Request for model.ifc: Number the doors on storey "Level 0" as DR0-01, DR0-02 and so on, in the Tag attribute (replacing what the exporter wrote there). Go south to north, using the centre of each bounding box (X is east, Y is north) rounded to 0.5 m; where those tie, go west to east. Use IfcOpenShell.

First a look at what the model holds.

```python
import ifcopenshell
import ifcopenshell.util.element
import ifcopenshell.util.placement

model = ifcopenshell.open("model.ifc")
print(model.schema)
storey = next(s for s in model.by_type("IfcBuildingStorey") if s.Name == "Level 0")
doors = [e for e in ifcopenshell.util.element.get_decomposition(storey) if e.is_a("IfcDoor")]
for e in sorted(doors, key=lambda e: e.id()):
    origin = ifcopenshell.util.placement.get_local_placement(e.ObjectPlacement)[:3, 3]
    print(e.id(), e.Tag, e.Name, origin.round(2) + 0.0, sep=" | ")
```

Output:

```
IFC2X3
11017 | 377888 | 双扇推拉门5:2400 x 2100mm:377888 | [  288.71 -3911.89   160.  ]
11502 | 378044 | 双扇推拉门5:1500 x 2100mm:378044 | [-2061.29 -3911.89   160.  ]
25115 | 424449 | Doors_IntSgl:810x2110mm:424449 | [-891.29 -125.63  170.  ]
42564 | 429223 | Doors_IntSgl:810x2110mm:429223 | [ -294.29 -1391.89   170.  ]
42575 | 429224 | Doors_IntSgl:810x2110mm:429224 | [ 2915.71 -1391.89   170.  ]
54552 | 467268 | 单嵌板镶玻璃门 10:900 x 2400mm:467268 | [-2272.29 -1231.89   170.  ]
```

```python
import ifcopenshell
import ifcopenshell.geom
import ifcopenshell.util.element
import ifcopenshell.util.shape

model = ifcopenshell.open("model.ifc")
settings = ifcopenshell.geom.settings()
settings.set("use-world-coords", True)


def centre(element):
    shape = ifcopenshell.geom.create_shape(settings, element)
    return ifcopenshell.util.shape.get_bbox_centroid(shape.geometry)


storey = next(s for s in model.by_type("IfcBuildingStorey") if s.Name == "Level 0")
doors = [e for e in ifcopenshell.util.element.get_decomposition(storey) if e.is_a("IfcDoor")]

# Insertion points can sit at a corner or the storey origin, so sort by the geometry (in metres).
centres = {e: centre(e) for e in doors}
doors.sort(key=lambda e: (round(centres[e][1] / 0.5), centres[e][0]))

for i, e in enumerate(doors, start=1):
    number = f"DR0-{i:02d}"
    e.Tag = number
    print(e.id(), number)

model.write("model_v2.ifc")
```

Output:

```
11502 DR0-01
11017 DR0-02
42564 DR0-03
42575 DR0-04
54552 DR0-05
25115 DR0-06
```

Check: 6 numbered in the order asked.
